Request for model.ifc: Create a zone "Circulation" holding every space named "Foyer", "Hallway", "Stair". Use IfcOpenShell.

First a look at what the model holds.

```python
import ifcopenshell

model = ifcopenshell.open("model.ifc")
print(model.schema)
seen = {}
for space in model.by_type("IfcSpace"):
    seen[space.LongName] = seen.get(space.LongName, 0) + 1
for name, count in sorted(seen.items(), key=str):
    print(count, "x", name)
print("zones:", [z.Name for z in model.by_type("IfcZone")][:20])
```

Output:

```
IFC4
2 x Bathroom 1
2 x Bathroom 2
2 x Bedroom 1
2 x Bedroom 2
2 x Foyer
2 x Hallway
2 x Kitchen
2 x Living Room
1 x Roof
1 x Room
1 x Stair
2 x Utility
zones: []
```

```python
import ifcopenshell
import ifcopenshell.api.group
import ifcopenshell.api.root

model = ifcopenshell.open("model.ifc")

names = {"Foyer", "Hallway", "Stair"}
spaces = [s for s in model.by_type("IfcSpace") if s.LongName in names]

zone = ifcopenshell.api.root.create_entity(model, ifc_class="IfcZone", name="Circulation")
ifcopenshell.api.group.assign_group(model, products=spaces, group=zone)
print(len(spaces), "spaces in", zone.Name)

model.write("model_rev.ifc")
```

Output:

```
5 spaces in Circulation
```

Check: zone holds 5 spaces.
